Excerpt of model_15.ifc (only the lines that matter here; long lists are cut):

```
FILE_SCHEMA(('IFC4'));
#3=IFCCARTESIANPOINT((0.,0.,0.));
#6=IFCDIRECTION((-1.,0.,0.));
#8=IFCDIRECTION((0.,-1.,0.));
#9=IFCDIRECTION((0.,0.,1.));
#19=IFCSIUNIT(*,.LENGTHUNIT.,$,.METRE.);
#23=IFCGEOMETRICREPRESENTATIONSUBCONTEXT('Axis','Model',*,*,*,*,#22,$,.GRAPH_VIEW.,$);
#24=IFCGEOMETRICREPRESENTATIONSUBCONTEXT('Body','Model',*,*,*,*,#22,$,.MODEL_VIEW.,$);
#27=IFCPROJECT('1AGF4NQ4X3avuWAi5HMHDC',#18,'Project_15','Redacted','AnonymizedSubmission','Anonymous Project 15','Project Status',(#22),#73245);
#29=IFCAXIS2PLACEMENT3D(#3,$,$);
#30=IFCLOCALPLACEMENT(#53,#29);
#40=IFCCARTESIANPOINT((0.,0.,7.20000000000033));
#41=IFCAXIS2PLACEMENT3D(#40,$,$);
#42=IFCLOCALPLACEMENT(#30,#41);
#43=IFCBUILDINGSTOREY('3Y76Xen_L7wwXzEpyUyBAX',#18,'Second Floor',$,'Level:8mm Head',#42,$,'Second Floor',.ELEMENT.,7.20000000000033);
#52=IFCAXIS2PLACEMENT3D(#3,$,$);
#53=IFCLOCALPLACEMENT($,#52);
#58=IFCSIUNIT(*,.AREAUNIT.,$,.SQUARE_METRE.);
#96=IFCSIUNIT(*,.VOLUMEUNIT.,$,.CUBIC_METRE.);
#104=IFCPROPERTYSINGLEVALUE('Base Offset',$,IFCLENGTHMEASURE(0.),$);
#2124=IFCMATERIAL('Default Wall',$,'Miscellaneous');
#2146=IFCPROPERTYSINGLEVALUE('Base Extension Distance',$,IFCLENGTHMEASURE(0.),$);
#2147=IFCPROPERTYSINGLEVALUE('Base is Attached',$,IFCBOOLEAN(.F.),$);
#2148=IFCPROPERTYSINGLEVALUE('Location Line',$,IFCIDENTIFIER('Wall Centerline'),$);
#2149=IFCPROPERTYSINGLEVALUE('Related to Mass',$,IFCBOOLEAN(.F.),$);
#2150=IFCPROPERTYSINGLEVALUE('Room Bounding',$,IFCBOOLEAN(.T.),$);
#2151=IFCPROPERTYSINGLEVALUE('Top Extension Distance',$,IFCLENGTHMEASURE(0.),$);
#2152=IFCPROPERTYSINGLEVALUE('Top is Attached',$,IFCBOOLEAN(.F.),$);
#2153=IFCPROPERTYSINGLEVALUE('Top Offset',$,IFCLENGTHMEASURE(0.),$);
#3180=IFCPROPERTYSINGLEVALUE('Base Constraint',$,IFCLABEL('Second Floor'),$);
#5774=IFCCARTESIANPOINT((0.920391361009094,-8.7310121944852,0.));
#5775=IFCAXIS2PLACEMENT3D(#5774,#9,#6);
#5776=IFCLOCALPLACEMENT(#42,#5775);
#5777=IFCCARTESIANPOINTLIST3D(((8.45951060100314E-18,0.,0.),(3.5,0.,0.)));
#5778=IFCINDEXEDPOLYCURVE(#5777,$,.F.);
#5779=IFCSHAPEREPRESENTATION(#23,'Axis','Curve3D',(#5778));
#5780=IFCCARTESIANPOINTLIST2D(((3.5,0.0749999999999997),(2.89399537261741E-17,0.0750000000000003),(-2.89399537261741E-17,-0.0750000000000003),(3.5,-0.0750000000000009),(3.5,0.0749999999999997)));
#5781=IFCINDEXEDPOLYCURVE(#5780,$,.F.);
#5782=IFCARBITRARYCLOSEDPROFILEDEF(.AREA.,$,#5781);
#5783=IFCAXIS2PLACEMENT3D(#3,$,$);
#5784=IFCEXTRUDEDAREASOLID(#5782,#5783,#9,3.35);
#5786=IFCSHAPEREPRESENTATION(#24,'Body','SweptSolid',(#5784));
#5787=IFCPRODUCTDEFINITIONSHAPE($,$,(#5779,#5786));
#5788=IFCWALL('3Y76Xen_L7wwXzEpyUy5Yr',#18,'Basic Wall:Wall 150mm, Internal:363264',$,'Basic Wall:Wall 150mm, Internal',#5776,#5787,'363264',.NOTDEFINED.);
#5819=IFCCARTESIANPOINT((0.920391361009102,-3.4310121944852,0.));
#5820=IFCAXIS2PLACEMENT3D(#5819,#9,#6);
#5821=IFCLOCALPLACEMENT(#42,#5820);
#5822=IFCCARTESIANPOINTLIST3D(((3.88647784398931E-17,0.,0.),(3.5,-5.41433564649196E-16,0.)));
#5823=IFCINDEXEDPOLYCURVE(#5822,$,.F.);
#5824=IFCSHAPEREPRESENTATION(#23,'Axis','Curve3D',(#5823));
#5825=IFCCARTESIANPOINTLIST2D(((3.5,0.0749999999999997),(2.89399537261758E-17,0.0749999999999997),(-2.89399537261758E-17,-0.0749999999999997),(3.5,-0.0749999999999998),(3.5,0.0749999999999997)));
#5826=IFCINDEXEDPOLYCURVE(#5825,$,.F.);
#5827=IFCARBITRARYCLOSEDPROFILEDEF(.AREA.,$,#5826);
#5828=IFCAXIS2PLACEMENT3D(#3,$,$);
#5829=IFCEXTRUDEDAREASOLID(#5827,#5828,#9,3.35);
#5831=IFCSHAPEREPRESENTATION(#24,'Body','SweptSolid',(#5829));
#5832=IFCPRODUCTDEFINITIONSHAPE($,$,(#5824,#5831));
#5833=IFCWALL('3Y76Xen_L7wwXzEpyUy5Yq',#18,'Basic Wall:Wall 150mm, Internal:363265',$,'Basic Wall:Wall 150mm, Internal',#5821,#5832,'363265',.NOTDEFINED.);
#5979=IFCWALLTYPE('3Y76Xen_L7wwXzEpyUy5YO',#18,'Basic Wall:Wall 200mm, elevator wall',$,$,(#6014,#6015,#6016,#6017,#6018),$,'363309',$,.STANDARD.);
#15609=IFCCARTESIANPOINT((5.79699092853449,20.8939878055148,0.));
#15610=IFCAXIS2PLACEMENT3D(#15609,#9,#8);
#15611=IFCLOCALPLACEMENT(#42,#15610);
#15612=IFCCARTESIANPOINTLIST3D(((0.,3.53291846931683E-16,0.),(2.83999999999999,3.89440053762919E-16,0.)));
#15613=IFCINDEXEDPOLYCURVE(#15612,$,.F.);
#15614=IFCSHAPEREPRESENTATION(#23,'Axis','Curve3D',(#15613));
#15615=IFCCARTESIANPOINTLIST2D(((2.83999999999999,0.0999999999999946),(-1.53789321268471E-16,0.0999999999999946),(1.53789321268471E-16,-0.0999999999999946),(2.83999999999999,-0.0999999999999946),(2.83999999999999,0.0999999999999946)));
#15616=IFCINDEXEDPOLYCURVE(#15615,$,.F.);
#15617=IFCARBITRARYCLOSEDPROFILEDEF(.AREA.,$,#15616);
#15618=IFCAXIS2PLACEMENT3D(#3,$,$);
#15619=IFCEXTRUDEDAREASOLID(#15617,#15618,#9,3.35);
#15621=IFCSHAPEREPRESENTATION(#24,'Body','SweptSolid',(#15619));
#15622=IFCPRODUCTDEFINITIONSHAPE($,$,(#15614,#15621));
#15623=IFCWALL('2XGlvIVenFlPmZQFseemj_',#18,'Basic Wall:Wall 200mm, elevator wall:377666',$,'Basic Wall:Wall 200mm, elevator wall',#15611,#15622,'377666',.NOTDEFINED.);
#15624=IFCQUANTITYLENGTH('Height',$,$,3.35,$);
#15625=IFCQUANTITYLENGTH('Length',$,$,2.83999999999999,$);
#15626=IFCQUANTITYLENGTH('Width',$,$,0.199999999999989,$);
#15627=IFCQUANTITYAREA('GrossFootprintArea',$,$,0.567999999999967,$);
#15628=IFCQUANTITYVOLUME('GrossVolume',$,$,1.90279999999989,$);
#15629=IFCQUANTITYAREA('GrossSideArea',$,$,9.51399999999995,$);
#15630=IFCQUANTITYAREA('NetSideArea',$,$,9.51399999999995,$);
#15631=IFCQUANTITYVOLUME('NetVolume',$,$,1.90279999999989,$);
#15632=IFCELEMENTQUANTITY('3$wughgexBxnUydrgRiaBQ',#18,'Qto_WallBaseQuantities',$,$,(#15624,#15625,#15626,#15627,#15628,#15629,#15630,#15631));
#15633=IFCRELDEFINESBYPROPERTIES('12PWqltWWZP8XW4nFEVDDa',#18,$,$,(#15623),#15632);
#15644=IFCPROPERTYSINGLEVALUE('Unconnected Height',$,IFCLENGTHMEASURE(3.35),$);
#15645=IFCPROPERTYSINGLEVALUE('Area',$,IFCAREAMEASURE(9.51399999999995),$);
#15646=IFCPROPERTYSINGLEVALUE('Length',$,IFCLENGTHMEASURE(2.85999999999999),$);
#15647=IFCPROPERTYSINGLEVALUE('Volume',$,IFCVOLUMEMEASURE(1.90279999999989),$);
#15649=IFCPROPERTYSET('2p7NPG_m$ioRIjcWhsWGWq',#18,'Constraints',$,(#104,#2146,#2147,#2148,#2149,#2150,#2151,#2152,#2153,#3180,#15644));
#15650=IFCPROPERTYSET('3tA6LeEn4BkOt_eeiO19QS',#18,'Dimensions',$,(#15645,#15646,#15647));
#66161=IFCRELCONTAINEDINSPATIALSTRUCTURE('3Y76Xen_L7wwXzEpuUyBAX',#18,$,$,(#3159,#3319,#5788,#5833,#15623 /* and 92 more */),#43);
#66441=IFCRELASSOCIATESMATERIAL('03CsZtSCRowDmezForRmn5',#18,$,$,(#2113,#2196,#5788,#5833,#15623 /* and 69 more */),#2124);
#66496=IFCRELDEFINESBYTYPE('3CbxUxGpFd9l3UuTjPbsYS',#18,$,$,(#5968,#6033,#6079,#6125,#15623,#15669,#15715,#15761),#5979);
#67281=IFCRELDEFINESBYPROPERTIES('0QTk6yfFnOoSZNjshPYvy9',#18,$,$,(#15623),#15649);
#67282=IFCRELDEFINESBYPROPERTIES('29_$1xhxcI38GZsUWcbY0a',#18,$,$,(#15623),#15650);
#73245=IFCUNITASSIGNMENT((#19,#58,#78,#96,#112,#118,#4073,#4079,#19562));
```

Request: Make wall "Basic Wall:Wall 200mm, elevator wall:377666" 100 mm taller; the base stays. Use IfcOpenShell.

```python
import ifcopenshell
import ifcopenshell.api.pset
import ifcopenshell.geom
import ifcopenshell.util.element
import ifcopenshell.util.representation
import ifcopenshell.util.shape
import ifcopenshell.util.unit

model = ifcopenshell.open("model_15.ifc")
unit_scale = ifcopenshell.util.unit.calculate_unit_scale(model)
area_scale = ifcopenshell.util.unit.calculate_unit_scale(model, "AREAUNIT")
volume_scale = ifcopenshell.util.unit.calculate_unit_scale(model, "VOLUMEUNIT")
settings = ifcopenshell.geom.settings()


def volume(element):
    """Net volume in cubic metres, openings subtracted."""
    shape = ifcopenshell.geom.create_shape(settings, element)
    return ifcopenshell.util.shape.get_volume(shape.geometry)


wall = model.by_guid("2XGlvIVenFlPmZQFseemj_")
before = volume(wall)

body = ifcopenshell.util.representation.get_representation(wall, "Model", "Body")
solid = body.Items[0]
old_height = solid.Depth
solid.Depth += 0.1
after = volume(wall)
thickness = 0.2  # wall thickness in metres

# Update the stored height, areas and volumes.
qto = model.by_id(ifcopenshell.util.element.get_pset(wall, "Qto_WallBaseQuantities", should_inherit=False)["id"])
ifcopenshell.api.pset.edit_qto(model, qto=qto, properties={
    "Height": solid.Depth,
    "GrossVolume": ifcopenshell.util.element.get_pset(wall, "Qto_WallBaseQuantities", "GrossVolume") * solid.Depth / old_height,
    "GrossSideArea": ifcopenshell.util.element.get_pset(wall, "Qto_WallBaseQuantities", "GrossSideArea") * solid.Depth / old_height,
    "NetSideArea": after / thickness / area_scale,
    "NetVolume": after / volume_scale,
})
pset = model.by_id(ifcopenshell.util.element.get_pset(wall, "Constraints", should_inherit=False)["id"])
ifcopenshell.api.pset.edit_pset(model, pset=pset, properties={
    "Unconnected Height": model.create_entity("IfcLengthMeasure", solid.Depth),
})
pset = model.by_id(ifcopenshell.util.element.get_pset(wall, "Dimensions", should_inherit=False)["id"])
ifcopenshell.api.pset.edit_pset(model, pset=pset, properties={
    "Area": model.create_entity("IfcAreaMeasure", after / thickness / area_scale),
    "Volume": model.create_entity("IfcVolumeMeasure", after / volume_scale),
})

print(f"height {old_height:g} -> {solid.Depth:g}, volume {before:.3f} -> {after:.3f} m3")

model.write("model_15_updated.ifc")
```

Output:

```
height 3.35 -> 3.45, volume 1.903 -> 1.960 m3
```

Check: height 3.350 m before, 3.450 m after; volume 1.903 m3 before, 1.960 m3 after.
